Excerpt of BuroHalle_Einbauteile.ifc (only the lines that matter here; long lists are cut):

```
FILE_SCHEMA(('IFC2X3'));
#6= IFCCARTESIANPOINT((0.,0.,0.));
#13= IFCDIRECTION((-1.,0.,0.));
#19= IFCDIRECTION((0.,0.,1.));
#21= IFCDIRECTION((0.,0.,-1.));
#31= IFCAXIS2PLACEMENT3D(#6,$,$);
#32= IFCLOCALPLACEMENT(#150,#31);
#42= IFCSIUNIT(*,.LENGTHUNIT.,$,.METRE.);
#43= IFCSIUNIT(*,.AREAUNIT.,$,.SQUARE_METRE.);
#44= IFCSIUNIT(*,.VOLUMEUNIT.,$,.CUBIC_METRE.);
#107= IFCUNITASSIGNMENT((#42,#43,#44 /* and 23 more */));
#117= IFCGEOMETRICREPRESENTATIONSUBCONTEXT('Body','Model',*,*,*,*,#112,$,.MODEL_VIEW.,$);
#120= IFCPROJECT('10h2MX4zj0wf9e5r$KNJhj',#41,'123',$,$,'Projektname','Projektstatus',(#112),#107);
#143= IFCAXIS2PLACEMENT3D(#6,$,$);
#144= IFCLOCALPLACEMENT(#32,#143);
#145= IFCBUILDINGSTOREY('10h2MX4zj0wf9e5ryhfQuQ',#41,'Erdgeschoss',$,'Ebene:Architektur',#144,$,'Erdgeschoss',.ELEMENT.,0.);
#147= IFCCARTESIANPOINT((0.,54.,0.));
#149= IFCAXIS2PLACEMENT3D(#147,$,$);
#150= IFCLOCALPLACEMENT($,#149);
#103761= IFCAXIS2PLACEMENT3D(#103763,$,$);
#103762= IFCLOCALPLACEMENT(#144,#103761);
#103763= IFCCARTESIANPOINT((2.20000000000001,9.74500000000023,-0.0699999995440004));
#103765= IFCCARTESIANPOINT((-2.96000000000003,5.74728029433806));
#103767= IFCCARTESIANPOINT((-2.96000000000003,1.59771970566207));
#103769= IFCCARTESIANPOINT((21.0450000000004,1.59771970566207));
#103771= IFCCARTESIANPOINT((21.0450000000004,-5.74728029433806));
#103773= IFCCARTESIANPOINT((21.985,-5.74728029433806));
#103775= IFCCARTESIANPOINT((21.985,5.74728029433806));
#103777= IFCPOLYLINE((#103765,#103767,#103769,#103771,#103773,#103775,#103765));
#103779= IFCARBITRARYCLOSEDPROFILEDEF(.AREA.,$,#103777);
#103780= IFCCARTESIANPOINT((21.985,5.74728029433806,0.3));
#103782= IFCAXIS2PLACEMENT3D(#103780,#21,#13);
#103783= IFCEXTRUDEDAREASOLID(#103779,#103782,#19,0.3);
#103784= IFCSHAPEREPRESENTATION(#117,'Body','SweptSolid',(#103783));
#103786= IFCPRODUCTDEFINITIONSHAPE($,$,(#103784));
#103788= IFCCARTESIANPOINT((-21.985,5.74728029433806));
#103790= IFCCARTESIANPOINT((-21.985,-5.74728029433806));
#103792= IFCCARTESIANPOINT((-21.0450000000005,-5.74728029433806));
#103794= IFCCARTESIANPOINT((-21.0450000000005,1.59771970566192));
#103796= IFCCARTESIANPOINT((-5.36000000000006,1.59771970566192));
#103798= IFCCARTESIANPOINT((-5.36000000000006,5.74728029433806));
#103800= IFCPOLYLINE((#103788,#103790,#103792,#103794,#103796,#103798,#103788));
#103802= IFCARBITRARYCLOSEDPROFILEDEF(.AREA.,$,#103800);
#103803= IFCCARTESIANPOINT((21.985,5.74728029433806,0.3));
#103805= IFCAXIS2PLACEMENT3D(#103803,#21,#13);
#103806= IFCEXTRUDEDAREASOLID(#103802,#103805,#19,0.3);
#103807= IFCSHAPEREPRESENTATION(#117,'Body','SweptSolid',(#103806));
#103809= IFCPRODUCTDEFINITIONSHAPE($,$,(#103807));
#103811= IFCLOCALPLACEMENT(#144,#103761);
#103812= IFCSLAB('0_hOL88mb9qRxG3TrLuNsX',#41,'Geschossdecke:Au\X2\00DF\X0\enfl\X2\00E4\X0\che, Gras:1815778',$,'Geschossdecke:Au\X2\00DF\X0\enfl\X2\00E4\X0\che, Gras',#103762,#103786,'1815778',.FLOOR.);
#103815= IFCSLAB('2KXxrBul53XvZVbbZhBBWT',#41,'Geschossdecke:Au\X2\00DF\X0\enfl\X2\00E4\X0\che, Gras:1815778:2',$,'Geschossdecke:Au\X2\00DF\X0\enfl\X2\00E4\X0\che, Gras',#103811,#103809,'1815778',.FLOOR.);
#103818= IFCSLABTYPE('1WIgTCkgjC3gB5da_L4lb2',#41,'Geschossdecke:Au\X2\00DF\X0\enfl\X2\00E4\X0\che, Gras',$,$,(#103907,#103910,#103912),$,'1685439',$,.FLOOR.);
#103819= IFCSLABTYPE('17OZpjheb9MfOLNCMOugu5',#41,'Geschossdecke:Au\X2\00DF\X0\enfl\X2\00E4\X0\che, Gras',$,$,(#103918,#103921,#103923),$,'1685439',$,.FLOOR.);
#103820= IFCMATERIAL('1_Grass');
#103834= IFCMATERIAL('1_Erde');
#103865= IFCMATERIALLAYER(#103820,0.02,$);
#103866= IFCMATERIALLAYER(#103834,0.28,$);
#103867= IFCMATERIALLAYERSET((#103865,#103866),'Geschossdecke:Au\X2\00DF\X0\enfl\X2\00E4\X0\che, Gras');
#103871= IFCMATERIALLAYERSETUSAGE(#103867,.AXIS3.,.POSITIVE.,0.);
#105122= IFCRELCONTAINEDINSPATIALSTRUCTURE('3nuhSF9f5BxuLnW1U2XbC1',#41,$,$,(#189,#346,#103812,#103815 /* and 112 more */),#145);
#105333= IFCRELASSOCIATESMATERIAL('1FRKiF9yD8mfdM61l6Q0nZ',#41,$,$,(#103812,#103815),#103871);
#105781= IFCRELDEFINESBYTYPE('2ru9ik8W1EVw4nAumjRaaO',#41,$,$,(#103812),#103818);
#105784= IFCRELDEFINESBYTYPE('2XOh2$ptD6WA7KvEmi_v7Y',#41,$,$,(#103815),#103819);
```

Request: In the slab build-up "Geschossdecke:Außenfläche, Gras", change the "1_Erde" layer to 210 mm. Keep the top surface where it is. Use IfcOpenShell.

```python
import ifcopenshell
import ifcopenshell.util.element
import ifcopenshell.util.representation

model = ifcopenshell.open("BuroHalle_Einbauteile.ifc")

layer_set = model.by_id(103867)
layer = next(l for l in layer_set.MaterialLayers if l.Material and l.Material.Name == "1_Erde")
change = 0.21 - layer.LayerThickness
layer.LayerThickness += change

# The layer set is shared, so every slab that uses it gets the new thickness.
slabs = [e for e in ifcopenshell.util.element.get_elements_by_material(model, layer_set) if e.is_a("IfcSlab")]
for slab in sorted(slabs, key=lambda e: e.id()):
    body = ifcopenshell.util.representation.get_representation(slab, "Model", "Body")
    solid = body.Items[0]
    old_depth = solid.Depth
    solid.Depth += change
    print(slab.id(), f"{old_depth:g} -> {solid.Depth:g}")

# The layers are counted up from the underside, which has moved.
for usage in {ifcopenshell.util.element.get_material(slab) for slab in slabs}:
    usage.OffsetFromReferenceLine -= change

model.write("BuroHalle_Einbauteile_edited.ifc")
```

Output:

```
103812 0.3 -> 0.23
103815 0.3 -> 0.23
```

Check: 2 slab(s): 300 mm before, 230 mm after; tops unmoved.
